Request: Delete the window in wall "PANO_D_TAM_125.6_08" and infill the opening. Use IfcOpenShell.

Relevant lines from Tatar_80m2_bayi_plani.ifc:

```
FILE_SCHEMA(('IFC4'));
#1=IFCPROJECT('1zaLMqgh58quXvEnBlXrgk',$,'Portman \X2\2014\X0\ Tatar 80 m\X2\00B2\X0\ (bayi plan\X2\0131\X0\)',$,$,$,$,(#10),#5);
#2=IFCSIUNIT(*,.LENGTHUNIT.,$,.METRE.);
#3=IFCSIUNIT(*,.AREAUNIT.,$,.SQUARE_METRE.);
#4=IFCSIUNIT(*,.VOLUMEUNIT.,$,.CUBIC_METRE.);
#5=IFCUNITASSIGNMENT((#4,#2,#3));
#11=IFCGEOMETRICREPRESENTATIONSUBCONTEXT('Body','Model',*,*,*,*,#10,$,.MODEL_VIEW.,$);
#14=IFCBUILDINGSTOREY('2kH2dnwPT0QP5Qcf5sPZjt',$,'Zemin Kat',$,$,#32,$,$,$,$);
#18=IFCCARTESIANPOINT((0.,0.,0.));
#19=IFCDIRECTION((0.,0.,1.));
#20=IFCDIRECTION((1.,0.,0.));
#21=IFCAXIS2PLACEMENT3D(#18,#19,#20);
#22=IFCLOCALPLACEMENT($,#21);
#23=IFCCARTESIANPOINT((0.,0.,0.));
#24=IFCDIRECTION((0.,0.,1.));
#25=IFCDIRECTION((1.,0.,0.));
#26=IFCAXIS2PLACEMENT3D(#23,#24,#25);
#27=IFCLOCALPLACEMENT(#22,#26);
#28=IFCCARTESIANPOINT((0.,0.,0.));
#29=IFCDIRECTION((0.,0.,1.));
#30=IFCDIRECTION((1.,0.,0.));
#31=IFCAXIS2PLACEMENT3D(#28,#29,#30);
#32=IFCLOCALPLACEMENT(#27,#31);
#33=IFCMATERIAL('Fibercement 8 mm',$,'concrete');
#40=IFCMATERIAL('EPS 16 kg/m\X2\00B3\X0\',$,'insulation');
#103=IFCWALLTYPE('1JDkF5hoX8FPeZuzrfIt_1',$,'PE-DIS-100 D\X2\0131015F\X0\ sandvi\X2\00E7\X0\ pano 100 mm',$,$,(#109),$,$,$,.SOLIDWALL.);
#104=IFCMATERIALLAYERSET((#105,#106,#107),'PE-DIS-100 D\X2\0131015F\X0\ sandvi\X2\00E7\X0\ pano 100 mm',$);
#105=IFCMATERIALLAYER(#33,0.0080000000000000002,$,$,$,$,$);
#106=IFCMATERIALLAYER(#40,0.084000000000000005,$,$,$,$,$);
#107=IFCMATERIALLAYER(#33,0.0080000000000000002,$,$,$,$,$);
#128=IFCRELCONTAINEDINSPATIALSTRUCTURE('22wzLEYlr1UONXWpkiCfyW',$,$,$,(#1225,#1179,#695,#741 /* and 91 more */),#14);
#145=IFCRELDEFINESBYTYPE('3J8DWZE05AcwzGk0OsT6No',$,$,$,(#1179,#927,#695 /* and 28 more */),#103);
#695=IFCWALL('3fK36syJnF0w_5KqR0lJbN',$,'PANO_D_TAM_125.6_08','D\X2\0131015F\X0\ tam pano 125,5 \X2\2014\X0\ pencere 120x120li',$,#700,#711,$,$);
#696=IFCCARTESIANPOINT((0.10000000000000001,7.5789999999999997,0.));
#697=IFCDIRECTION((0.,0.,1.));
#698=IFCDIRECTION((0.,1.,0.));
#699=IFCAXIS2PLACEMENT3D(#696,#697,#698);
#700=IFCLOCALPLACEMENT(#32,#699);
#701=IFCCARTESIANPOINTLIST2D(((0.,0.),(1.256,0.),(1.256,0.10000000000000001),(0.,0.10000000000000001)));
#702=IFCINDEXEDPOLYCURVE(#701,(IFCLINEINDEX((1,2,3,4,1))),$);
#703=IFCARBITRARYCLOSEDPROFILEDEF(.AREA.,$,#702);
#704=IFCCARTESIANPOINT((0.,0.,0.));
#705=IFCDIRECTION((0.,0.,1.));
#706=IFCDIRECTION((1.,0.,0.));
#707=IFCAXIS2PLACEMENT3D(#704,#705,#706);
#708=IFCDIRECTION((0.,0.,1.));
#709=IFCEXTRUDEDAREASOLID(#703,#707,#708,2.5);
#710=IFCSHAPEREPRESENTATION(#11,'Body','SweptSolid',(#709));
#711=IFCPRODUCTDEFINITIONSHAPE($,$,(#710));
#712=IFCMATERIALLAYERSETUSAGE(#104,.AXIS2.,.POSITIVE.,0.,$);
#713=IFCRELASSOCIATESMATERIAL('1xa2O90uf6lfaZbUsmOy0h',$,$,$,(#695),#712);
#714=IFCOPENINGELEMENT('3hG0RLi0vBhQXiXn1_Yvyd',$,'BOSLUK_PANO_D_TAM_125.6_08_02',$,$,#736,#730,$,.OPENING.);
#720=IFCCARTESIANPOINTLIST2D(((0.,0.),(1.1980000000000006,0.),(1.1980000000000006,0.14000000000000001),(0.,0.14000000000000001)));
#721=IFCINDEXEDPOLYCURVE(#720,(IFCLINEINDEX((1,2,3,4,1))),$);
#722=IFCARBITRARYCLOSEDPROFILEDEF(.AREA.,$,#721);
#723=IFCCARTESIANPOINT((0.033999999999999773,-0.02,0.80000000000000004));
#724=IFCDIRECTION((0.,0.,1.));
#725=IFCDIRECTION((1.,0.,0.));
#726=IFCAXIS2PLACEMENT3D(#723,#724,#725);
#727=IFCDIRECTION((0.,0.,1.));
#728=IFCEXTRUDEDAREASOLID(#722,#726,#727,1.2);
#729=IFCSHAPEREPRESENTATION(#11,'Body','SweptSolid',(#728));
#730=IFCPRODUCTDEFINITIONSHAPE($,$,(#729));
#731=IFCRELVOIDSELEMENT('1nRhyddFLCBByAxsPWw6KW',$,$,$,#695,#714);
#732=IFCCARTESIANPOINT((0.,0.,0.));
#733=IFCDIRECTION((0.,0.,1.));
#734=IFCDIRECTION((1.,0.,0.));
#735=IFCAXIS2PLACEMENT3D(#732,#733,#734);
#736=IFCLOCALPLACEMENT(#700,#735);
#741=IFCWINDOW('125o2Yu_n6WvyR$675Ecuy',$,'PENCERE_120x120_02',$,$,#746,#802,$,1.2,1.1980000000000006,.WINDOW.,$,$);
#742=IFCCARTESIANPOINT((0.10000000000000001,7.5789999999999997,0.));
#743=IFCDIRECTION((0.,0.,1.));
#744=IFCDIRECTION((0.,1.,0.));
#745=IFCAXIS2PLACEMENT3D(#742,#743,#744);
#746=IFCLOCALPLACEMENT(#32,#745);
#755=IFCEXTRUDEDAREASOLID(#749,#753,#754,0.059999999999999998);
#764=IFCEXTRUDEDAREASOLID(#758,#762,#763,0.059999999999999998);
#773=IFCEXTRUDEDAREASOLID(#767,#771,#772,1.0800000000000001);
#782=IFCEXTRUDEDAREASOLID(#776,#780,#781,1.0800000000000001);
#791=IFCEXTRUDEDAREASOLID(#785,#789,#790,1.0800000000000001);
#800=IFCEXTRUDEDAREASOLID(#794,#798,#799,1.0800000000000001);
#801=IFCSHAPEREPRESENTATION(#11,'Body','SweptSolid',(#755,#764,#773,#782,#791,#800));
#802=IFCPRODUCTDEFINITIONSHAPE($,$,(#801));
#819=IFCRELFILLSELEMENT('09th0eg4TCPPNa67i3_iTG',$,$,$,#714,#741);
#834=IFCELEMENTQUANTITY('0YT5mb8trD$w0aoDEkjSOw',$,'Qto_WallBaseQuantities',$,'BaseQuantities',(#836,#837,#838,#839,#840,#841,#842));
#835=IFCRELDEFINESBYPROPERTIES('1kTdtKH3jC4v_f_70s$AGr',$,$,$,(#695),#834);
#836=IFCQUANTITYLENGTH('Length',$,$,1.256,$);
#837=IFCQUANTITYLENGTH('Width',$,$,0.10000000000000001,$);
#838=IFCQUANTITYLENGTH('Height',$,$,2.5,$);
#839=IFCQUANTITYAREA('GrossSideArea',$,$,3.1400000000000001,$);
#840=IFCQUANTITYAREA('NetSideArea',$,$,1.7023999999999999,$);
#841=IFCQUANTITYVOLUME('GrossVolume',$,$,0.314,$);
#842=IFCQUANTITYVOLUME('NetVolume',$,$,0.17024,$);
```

```python
import ifcopenshell
import ifcopenshell.api.feature
import ifcopenshell.api.pset
import ifcopenshell.api.root
import ifcopenshell.geom
import ifcopenshell.util.element
import ifcopenshell.util.shape
import ifcopenshell.util.unit

model = ifcopenshell.open("Tatar_80m2_bayi_plani.ifc")
area_scale = ifcopenshell.util.unit.calculate_unit_scale(model, "AREAUNIT")
volume_scale = ifcopenshell.util.unit.calculate_unit_scale(model, "VOLUMEUNIT")
settings = ifcopenshell.geom.settings()


def volume(element):
    """Net volume in cubic metres, openings subtracted."""
    shape = ifcopenshell.geom.create_shape(settings, element)
    return ifcopenshell.util.shape.get_volume(shape.geometry)


window = model.by_id(741)
opening = window.FillsVoids[0].RelatingOpeningElement
wall = opening.VoidsElements[0].RelatingBuildingElement
before = volume(wall)

ifcopenshell.api.root.remove_product(model, product=window)
ifcopenshell.api.feature.remove_feature(model, feature=opening)

after = volume(wall)
thickness = 0.1  # wall thickness in metres

# Update the wall's stored quantities.
qto = model.by_id(ifcopenshell.util.element.get_pset(wall, "Qto_WallBaseQuantities", should_inherit=False)["id"])
ifcopenshell.api.pset.edit_qto(model, qto=qto, properties={
    "NetSideArea": after / thickness / area_scale,
    "NetVolume": after / volume_scale,
})

print(f"wall volume {before:.3f} -> {after:.3f} m3")

model.write("Tatar_80m2_bayi_plani_rev.ifc")
```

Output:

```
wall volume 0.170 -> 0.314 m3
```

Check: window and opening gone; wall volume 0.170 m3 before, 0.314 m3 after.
